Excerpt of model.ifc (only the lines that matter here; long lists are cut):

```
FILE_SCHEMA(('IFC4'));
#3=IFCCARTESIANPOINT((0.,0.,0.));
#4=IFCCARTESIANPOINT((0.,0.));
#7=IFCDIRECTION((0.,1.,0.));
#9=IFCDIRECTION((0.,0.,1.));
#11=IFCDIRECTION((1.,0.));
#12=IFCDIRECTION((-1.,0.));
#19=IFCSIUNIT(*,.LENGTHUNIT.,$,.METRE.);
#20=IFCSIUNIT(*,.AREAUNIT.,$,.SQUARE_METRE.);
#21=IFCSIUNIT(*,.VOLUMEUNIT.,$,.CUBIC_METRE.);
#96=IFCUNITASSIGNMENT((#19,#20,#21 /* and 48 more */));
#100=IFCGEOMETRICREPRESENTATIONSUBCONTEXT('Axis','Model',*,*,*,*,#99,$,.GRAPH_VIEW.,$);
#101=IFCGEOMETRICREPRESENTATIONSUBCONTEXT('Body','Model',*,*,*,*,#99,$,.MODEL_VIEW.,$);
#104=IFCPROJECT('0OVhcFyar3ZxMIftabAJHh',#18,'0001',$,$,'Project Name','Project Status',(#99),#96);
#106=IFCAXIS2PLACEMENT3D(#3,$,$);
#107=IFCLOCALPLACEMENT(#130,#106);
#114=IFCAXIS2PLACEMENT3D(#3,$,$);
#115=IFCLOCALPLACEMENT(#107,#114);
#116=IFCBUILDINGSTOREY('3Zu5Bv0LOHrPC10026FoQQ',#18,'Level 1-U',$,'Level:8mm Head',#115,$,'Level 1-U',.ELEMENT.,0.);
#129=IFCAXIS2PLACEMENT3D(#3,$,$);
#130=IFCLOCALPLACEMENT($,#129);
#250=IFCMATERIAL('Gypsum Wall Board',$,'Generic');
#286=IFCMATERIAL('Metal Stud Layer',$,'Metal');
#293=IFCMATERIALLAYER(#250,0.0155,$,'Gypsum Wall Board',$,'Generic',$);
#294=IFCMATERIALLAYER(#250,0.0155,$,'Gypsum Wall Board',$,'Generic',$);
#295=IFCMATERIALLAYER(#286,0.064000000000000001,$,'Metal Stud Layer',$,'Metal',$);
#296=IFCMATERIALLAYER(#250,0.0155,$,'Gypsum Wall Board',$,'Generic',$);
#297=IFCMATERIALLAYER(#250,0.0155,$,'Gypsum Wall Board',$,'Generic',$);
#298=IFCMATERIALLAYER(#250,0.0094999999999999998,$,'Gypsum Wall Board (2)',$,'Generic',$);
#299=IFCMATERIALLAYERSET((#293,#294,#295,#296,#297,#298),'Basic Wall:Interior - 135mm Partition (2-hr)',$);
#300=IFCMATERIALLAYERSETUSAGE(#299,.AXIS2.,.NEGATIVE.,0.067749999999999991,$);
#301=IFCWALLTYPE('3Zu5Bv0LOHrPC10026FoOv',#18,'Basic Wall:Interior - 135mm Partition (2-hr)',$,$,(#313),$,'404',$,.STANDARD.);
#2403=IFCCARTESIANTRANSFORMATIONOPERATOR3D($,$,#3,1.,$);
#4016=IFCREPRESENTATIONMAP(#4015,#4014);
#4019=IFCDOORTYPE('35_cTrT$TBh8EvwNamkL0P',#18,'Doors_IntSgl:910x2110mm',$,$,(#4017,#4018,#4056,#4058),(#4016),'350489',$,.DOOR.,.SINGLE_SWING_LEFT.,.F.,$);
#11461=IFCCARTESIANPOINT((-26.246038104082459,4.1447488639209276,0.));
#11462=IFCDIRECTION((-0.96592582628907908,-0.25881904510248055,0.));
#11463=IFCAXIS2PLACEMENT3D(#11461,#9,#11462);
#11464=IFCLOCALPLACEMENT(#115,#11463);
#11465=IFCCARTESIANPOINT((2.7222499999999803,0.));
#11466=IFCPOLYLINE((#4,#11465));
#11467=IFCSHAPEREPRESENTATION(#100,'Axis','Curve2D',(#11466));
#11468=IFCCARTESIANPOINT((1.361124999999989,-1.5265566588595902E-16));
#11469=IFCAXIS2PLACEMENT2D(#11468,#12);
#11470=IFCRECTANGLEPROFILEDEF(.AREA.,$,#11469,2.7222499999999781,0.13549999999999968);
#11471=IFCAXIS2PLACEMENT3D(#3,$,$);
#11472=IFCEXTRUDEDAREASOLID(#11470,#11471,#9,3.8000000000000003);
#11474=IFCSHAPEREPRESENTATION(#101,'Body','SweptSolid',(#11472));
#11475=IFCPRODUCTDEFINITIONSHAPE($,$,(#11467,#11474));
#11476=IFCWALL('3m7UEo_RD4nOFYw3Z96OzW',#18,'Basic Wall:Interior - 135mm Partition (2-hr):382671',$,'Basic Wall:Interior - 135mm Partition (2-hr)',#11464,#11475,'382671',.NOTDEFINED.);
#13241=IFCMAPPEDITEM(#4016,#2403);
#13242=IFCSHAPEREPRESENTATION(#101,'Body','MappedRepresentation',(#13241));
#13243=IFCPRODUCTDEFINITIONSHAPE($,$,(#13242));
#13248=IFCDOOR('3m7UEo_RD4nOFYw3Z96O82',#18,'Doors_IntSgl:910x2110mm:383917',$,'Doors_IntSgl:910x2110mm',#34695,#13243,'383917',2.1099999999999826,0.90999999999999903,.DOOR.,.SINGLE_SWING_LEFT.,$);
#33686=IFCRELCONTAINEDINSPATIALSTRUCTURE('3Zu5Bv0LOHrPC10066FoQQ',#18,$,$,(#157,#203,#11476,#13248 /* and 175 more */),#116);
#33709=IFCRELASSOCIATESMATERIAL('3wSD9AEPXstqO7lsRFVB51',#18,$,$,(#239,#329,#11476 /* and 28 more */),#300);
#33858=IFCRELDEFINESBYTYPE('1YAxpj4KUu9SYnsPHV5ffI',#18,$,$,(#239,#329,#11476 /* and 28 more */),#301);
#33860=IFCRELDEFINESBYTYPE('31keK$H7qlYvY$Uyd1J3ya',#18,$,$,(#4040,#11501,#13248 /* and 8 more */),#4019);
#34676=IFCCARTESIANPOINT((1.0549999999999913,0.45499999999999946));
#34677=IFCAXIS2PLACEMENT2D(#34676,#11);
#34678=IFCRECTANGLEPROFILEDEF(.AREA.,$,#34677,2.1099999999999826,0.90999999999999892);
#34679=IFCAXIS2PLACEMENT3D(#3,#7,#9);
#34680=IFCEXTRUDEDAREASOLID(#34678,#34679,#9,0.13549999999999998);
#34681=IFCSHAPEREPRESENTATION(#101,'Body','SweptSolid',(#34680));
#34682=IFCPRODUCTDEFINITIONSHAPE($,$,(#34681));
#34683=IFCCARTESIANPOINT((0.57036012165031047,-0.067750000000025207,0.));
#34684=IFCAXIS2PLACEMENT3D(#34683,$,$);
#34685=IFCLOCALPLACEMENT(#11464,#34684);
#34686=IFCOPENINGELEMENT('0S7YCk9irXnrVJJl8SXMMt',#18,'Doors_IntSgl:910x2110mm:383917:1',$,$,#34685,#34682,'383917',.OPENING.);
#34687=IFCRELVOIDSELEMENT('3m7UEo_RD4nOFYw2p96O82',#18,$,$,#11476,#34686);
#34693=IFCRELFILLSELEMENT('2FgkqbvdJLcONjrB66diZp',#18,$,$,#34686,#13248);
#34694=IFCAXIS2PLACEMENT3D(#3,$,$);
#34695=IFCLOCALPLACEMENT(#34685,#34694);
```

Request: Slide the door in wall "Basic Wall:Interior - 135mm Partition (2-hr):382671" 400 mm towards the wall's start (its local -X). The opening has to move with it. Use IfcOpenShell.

```python
import ifcopenshell
import ifcopenshell.api.geometry
import ifcopenshell.util.placement
import ifcopenshell.util.unit

model = ifcopenshell.open("model.ifc")
unit_scale = ifcopenshell.util.unit.calculate_unit_scale(model)

door = model.by_guid("3m7UEo_RD4nOFYw3Z96O82")
opening = door.FillsVoids[0].RelatingOpeningElement
wall = opening.VoidsElements[0].RelatingBuildingElement

wall_matrix = ifcopenshell.util.placement.get_local_placement(wall.ObjectPlacement)
shift = wall_matrix[:3, 0] * -0.4 / unit_scale
before = ifcopenshell.util.placement.get_local_placement(door.ObjectPlacement)[:3, 3].copy()

# The door is placed relative to its opening, so it follows when the opening moves.
matrix = ifcopenshell.util.placement.get_local_placement(opening.ObjectPlacement)
matrix[:3, 3] += shift
ifcopenshell.api.geometry.edit_object_placement(
    model, product=opening, matrix=matrix, is_si=False, should_transform_children=True
)

after = ifcopenshell.util.placement.get_local_placement(door.ObjectPlacement)[:3, 3]
print("door moved by", (after - before).round(3) + 0.0)

model.write("model-out.ifc")
```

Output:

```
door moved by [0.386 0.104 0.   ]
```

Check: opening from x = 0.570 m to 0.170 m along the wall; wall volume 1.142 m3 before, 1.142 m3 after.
